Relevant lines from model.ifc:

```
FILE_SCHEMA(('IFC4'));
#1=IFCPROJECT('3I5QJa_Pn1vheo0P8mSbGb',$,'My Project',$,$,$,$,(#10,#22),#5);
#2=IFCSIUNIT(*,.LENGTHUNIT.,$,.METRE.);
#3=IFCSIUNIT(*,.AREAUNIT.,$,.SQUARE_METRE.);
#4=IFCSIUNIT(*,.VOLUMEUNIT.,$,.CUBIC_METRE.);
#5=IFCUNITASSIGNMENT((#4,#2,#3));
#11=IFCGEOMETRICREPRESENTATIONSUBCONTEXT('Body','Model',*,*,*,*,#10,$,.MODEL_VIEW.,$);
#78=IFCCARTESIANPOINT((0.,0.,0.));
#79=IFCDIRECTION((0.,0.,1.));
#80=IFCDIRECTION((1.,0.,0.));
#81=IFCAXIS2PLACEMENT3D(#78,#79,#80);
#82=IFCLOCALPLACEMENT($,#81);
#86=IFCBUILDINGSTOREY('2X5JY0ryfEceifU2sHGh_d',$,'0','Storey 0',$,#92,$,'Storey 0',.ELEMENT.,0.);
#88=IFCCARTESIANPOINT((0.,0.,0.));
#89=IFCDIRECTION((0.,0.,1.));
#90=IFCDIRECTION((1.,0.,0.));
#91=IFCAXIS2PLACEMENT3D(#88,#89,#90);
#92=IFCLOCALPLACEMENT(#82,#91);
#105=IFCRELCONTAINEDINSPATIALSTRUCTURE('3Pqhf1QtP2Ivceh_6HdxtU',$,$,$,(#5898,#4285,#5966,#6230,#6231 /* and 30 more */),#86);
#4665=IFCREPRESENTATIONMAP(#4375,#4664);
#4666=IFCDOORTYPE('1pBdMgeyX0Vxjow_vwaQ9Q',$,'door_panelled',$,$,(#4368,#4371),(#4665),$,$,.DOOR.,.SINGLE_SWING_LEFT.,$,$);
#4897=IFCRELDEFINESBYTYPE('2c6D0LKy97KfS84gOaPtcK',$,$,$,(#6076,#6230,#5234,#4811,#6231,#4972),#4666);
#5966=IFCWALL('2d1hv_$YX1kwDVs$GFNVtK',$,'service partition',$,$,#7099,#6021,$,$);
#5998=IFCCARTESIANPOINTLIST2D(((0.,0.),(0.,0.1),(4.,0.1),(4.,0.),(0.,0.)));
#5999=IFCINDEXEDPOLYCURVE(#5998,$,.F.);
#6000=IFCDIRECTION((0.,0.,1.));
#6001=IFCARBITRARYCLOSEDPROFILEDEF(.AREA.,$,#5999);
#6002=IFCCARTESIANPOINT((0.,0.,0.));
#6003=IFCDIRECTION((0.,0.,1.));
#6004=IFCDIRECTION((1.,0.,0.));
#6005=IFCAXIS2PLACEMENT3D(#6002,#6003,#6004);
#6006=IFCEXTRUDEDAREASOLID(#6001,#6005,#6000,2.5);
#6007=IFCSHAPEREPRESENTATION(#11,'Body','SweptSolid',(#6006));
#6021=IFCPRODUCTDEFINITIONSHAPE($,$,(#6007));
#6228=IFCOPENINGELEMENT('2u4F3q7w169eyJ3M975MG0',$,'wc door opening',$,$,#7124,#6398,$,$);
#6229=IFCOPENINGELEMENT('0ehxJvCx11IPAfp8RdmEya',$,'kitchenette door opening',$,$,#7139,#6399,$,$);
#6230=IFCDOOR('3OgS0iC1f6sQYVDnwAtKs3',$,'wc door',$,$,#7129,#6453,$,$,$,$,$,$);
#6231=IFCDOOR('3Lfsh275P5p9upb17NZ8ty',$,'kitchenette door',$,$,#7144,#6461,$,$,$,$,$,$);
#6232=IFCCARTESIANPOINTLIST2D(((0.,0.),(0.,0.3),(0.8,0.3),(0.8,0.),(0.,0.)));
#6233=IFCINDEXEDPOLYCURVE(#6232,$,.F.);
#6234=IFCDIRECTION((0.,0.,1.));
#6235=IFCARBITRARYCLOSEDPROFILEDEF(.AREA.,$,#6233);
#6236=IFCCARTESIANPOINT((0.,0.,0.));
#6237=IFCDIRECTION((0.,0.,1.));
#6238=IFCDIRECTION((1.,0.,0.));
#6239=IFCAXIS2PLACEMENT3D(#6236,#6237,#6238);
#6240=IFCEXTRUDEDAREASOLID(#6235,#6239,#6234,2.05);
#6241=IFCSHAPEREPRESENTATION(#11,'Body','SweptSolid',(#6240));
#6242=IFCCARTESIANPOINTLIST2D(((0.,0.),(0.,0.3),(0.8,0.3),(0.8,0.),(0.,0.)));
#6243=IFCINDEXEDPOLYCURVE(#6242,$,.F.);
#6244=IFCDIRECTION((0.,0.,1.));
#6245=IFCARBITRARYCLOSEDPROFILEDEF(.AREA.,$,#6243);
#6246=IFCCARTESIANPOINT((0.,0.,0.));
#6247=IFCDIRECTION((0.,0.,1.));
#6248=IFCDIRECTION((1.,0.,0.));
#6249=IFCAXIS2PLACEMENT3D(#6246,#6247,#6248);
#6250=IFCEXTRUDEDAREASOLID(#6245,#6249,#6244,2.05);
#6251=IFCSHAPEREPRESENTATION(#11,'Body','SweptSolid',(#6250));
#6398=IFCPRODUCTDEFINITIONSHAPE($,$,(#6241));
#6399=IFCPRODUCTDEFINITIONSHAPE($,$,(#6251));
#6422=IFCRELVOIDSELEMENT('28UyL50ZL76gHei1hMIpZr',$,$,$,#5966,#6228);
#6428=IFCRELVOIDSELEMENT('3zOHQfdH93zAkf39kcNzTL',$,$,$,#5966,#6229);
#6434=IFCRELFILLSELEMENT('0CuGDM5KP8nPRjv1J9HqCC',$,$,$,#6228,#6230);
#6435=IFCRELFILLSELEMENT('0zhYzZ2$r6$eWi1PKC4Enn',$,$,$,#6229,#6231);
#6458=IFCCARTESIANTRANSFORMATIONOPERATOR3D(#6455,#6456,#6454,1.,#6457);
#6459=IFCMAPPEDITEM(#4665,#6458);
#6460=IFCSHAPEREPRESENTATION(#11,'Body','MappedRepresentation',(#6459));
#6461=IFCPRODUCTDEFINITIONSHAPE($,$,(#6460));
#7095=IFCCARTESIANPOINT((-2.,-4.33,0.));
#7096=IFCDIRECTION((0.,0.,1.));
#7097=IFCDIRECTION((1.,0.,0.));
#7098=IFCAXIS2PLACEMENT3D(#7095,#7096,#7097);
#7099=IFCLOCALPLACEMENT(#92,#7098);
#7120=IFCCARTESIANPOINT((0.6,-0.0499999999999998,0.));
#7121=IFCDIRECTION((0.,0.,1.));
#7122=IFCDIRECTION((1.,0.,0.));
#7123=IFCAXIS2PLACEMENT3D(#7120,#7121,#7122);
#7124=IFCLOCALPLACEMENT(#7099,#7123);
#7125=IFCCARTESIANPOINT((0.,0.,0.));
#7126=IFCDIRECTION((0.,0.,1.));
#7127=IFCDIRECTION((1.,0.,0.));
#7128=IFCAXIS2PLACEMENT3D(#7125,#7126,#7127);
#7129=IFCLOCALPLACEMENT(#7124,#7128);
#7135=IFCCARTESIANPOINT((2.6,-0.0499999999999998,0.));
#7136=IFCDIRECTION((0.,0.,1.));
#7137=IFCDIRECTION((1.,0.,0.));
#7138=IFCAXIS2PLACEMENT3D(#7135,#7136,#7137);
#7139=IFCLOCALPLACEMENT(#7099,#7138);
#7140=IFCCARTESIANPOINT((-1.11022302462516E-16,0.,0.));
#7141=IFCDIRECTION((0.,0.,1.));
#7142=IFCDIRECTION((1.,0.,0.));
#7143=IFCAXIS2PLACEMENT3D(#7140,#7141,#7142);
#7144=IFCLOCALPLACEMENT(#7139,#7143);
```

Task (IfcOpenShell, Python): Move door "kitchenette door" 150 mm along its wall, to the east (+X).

```python
import ifcopenshell
import ifcopenshell.api.geometry
import ifcopenshell.util.placement
import ifcopenshell.util.unit

model = ifcopenshell.open("model.ifc")
unit_scale = ifcopenshell.util.unit.calculate_unit_scale(model)

door = model.by_guid("3Lfsh275P5p9upb17NZ8ty")
opening = door.FillsVoids[0].RelatingOpeningElement
wall = opening.VoidsElements[0].RelatingBuildingElement

wall_matrix = ifcopenshell.util.placement.get_local_placement(wall.ObjectPlacement)
shift = wall_matrix[:3, 0] * 0.15 / unit_scale
before = ifcopenshell.util.placement.get_local_placement(door.ObjectPlacement)[:3, 3].copy()

# The door is placed relative to its opening, so it follows when the opening moves.
matrix = ifcopenshell.util.placement.get_local_placement(opening.ObjectPlacement)
matrix[:3, 3] += shift
ifcopenshell.api.geometry.edit_object_placement(
    model, product=opening, matrix=matrix, is_si=False, should_transform_children=True
)

after = ifcopenshell.util.placement.get_local_placement(door.ObjectPlacement)[:3, 3]
print("door moved by", (after - before).round(3) + 0.0)

model.write("model_v2.ifc")
```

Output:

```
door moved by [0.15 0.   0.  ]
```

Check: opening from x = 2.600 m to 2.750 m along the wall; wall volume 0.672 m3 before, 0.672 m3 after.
